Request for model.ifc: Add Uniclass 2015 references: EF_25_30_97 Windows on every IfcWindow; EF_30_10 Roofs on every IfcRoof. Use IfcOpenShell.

First a look at what the model holds.

```python
import ifcopenshell

model = ifcopenshell.open("model.ifc")
print(model.schema)
print("classifications:", [c.Name for c in model.by_type("IfcClassification")])
for ifc_class in ("IfcDoor", "IfcRoof", "IfcStair", "IfcWall", "IfcWindow"):
    print(ifc_class, len(model.by_type(ifc_class)))
```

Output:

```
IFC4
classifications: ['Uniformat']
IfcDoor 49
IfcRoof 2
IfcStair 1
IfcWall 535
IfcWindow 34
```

```python
import ifcopenshell
import ifcopenshell.api.classification

model = ifcopenshell.open("model.ifc")

system = ifcopenshell.api.classification.add_classification(model, classification="Uniclass 2015")

codes = {
    "IfcWindow": ("EF_25_30_97", "Windows"),
    "IfcRoof": ("EF_30_10", "Roofs"),
}
for ifc_class, (code, name) in codes.items():
    products = model.by_type(ifc_class)
    ifcopenshell.api.classification.add_reference(
        model, products=products, classification=system, identification=code, name=name
    )
    print(code, len(products))

model.write("model-out.ifc")
```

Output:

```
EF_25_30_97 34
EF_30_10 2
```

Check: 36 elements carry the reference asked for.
